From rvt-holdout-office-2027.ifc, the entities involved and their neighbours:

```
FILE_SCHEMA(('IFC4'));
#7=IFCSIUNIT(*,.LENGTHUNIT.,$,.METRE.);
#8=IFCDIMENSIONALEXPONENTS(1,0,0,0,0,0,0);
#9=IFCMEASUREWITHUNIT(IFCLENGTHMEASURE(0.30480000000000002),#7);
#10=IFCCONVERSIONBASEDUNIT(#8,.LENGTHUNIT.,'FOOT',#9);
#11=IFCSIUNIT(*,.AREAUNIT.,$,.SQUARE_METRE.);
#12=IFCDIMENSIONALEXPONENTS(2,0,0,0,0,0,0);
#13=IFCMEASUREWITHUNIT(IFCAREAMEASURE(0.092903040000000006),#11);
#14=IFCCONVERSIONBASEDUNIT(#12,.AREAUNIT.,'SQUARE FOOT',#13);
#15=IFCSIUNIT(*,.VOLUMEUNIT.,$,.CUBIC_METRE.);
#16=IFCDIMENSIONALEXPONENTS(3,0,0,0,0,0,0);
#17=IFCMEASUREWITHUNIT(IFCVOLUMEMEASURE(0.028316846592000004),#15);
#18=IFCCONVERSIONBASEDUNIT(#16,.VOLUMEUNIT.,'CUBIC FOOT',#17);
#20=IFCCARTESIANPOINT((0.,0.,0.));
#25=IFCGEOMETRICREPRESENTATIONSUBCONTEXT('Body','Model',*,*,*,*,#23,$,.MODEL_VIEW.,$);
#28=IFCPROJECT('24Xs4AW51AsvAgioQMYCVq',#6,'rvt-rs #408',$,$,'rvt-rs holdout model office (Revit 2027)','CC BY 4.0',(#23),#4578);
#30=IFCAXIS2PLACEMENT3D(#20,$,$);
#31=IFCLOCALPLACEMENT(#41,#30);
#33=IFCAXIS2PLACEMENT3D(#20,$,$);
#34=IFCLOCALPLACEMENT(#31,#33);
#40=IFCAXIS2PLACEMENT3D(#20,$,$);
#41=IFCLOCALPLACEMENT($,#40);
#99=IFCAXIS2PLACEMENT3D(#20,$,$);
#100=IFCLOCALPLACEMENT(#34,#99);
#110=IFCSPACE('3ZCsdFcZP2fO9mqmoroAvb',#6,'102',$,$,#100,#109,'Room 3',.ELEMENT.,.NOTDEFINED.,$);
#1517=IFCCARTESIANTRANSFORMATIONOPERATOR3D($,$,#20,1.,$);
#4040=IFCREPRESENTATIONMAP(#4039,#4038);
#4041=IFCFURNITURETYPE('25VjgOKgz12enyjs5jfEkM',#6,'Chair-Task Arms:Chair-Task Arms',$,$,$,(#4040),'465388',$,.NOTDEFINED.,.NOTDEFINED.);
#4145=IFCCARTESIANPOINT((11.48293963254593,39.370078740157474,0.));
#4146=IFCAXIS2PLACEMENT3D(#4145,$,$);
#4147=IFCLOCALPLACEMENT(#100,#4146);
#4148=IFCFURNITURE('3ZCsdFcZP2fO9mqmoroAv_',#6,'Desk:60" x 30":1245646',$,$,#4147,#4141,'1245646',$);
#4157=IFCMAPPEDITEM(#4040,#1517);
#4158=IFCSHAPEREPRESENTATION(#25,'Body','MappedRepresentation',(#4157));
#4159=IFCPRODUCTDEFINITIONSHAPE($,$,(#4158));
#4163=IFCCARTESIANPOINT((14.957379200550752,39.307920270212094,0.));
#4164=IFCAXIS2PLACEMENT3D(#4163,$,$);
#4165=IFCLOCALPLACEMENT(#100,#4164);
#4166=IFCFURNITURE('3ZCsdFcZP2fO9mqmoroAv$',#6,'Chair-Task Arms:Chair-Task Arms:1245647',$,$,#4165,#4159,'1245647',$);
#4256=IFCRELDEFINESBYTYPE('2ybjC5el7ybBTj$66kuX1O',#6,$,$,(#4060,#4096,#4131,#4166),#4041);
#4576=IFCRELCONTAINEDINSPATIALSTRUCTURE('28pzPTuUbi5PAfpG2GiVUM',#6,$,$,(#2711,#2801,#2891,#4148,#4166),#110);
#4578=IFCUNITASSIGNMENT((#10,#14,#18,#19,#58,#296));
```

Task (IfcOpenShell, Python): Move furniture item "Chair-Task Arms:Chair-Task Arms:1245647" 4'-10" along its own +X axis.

```python
import ifcopenshell
import ifcopenshell.api.geometry
import ifcopenshell.util.placement
import ifcopenshell.util.unit

model = ifcopenshell.open("rvt-holdout-office-2027.ifc")
unit_scale = ifcopenshell.util.unit.calculate_unit_scale(model)

item = model.by_guid("3ZCsdFcZP2fO9mqmoroAv$")
matrix = ifcopenshell.util.placement.get_local_placement(item.ObjectPlacement)
matrix[:3, 3] += matrix[:3, 0] * 58 * 0.0254 / unit_scale
ifcopenshell.api.geometry.edit_object_placement(model, product=item, matrix=matrix, is_si=False)

print(ifcopenshell.util.placement.get_local_placement(item.ObjectPlacement).round(3) + 0.0)

model.write("rvt-holdout-office-2027_edited.ifc")
```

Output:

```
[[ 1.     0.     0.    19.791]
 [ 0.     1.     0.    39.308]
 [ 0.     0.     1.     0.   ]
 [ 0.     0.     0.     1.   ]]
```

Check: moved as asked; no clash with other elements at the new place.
